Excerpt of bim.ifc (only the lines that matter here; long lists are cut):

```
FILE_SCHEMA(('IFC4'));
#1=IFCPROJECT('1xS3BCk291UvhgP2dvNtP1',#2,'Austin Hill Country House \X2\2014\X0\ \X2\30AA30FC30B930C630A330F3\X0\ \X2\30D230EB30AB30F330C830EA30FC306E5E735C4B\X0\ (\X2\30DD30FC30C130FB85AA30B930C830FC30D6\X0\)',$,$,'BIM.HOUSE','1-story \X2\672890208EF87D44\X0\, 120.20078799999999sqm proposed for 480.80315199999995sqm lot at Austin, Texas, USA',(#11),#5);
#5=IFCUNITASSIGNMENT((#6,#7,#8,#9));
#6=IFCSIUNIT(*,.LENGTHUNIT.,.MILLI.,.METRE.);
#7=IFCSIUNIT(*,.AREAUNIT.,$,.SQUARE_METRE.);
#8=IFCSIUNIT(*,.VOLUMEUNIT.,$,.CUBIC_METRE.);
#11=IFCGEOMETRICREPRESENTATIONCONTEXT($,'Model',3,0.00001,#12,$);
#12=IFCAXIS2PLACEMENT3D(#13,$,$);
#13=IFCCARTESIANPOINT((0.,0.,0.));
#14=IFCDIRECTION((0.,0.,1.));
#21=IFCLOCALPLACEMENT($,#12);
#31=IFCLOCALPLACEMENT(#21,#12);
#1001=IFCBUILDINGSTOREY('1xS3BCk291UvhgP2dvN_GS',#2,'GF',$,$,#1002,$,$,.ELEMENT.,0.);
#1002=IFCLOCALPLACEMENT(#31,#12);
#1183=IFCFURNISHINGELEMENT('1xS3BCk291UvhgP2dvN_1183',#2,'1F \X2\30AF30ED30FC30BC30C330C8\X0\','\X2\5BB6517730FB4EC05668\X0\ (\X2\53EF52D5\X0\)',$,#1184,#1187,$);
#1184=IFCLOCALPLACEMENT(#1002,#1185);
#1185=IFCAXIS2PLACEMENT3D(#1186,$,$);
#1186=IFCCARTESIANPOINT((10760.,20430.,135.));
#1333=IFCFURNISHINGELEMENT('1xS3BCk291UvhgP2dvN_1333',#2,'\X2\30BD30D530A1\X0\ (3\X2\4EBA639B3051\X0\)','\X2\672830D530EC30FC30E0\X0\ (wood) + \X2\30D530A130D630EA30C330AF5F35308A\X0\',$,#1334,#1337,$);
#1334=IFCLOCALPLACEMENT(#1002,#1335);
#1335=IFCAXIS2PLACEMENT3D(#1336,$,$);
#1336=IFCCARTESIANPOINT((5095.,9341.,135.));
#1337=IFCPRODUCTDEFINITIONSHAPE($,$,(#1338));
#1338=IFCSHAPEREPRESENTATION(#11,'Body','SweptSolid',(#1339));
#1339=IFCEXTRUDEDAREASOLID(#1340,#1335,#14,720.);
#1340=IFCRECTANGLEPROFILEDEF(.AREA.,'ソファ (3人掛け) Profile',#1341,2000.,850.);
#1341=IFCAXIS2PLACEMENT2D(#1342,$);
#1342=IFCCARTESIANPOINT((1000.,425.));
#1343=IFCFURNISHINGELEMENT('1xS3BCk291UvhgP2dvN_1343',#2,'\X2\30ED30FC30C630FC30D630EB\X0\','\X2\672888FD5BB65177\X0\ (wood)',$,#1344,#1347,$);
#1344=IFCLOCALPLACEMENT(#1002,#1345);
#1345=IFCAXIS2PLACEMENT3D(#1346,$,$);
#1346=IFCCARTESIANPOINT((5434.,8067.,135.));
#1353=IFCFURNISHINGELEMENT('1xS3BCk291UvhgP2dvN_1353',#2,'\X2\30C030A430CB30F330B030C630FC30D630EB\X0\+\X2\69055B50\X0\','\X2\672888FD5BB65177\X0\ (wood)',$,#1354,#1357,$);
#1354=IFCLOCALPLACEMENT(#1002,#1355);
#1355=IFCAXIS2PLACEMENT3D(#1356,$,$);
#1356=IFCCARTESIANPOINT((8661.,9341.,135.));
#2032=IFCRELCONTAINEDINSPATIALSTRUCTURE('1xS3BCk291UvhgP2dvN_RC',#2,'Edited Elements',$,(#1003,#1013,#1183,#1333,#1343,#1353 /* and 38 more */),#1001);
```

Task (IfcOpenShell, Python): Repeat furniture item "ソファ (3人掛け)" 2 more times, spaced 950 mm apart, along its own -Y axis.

```python
import ifcopenshell
import ifcopenshell.api.geometry
import ifcopenshell.api.root
import ifcopenshell.util.element
import ifcopenshell.util.placement
import ifcopenshell.util.unit

model = ifcopenshell.open("bim.ifc")
unit_scale = ifcopenshell.util.unit.calculate_unit_scale(model)


def reuse_history(source, copy):
    """copy_class also copies each property set's owner history, people and application; keep the originals."""
    for rel in copy.IsDefinedBy:
        if rel.is_a("IfcRelDefinesByProperties") and (history := rel.RelatingPropertyDefinition.OwnerHistory):
            rel.RelatingPropertyDefinition.OwnerHistory = source.OwnerHistory
            ifcopenshell.util.element.remove_deep2(model, history)


source = model.by_guid("1xS3BCk291UvhgP2dvN_1333")
base = ifcopenshell.util.placement.get_local_placement(source.ObjectPlacement)
step = -base[:3, 1] * 0.95 / unit_scale

for i in range(1, 3):
    copy = ifcopenshell.api.root.copy_class(model, product=source)
    copy.Representation = ifcopenshell.util.element.copy_deep(
        model, source.Representation, exclude=["IfcGeometricRepresentationContext", "IfcRepresentationMap"]
    )
    reuse_history(source, copy)
    matrix = base.copy()
    matrix[:3, 3] += i * step
    print("added at", matrix[:3, 3].round(3) + 0.0)
    ifcopenshell.api.geometry.edit_object_placement(model, product=copy, matrix=matrix, is_si=False)

model.write("bim_rev.ifc")
```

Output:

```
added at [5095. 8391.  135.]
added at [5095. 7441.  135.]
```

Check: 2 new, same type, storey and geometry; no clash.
